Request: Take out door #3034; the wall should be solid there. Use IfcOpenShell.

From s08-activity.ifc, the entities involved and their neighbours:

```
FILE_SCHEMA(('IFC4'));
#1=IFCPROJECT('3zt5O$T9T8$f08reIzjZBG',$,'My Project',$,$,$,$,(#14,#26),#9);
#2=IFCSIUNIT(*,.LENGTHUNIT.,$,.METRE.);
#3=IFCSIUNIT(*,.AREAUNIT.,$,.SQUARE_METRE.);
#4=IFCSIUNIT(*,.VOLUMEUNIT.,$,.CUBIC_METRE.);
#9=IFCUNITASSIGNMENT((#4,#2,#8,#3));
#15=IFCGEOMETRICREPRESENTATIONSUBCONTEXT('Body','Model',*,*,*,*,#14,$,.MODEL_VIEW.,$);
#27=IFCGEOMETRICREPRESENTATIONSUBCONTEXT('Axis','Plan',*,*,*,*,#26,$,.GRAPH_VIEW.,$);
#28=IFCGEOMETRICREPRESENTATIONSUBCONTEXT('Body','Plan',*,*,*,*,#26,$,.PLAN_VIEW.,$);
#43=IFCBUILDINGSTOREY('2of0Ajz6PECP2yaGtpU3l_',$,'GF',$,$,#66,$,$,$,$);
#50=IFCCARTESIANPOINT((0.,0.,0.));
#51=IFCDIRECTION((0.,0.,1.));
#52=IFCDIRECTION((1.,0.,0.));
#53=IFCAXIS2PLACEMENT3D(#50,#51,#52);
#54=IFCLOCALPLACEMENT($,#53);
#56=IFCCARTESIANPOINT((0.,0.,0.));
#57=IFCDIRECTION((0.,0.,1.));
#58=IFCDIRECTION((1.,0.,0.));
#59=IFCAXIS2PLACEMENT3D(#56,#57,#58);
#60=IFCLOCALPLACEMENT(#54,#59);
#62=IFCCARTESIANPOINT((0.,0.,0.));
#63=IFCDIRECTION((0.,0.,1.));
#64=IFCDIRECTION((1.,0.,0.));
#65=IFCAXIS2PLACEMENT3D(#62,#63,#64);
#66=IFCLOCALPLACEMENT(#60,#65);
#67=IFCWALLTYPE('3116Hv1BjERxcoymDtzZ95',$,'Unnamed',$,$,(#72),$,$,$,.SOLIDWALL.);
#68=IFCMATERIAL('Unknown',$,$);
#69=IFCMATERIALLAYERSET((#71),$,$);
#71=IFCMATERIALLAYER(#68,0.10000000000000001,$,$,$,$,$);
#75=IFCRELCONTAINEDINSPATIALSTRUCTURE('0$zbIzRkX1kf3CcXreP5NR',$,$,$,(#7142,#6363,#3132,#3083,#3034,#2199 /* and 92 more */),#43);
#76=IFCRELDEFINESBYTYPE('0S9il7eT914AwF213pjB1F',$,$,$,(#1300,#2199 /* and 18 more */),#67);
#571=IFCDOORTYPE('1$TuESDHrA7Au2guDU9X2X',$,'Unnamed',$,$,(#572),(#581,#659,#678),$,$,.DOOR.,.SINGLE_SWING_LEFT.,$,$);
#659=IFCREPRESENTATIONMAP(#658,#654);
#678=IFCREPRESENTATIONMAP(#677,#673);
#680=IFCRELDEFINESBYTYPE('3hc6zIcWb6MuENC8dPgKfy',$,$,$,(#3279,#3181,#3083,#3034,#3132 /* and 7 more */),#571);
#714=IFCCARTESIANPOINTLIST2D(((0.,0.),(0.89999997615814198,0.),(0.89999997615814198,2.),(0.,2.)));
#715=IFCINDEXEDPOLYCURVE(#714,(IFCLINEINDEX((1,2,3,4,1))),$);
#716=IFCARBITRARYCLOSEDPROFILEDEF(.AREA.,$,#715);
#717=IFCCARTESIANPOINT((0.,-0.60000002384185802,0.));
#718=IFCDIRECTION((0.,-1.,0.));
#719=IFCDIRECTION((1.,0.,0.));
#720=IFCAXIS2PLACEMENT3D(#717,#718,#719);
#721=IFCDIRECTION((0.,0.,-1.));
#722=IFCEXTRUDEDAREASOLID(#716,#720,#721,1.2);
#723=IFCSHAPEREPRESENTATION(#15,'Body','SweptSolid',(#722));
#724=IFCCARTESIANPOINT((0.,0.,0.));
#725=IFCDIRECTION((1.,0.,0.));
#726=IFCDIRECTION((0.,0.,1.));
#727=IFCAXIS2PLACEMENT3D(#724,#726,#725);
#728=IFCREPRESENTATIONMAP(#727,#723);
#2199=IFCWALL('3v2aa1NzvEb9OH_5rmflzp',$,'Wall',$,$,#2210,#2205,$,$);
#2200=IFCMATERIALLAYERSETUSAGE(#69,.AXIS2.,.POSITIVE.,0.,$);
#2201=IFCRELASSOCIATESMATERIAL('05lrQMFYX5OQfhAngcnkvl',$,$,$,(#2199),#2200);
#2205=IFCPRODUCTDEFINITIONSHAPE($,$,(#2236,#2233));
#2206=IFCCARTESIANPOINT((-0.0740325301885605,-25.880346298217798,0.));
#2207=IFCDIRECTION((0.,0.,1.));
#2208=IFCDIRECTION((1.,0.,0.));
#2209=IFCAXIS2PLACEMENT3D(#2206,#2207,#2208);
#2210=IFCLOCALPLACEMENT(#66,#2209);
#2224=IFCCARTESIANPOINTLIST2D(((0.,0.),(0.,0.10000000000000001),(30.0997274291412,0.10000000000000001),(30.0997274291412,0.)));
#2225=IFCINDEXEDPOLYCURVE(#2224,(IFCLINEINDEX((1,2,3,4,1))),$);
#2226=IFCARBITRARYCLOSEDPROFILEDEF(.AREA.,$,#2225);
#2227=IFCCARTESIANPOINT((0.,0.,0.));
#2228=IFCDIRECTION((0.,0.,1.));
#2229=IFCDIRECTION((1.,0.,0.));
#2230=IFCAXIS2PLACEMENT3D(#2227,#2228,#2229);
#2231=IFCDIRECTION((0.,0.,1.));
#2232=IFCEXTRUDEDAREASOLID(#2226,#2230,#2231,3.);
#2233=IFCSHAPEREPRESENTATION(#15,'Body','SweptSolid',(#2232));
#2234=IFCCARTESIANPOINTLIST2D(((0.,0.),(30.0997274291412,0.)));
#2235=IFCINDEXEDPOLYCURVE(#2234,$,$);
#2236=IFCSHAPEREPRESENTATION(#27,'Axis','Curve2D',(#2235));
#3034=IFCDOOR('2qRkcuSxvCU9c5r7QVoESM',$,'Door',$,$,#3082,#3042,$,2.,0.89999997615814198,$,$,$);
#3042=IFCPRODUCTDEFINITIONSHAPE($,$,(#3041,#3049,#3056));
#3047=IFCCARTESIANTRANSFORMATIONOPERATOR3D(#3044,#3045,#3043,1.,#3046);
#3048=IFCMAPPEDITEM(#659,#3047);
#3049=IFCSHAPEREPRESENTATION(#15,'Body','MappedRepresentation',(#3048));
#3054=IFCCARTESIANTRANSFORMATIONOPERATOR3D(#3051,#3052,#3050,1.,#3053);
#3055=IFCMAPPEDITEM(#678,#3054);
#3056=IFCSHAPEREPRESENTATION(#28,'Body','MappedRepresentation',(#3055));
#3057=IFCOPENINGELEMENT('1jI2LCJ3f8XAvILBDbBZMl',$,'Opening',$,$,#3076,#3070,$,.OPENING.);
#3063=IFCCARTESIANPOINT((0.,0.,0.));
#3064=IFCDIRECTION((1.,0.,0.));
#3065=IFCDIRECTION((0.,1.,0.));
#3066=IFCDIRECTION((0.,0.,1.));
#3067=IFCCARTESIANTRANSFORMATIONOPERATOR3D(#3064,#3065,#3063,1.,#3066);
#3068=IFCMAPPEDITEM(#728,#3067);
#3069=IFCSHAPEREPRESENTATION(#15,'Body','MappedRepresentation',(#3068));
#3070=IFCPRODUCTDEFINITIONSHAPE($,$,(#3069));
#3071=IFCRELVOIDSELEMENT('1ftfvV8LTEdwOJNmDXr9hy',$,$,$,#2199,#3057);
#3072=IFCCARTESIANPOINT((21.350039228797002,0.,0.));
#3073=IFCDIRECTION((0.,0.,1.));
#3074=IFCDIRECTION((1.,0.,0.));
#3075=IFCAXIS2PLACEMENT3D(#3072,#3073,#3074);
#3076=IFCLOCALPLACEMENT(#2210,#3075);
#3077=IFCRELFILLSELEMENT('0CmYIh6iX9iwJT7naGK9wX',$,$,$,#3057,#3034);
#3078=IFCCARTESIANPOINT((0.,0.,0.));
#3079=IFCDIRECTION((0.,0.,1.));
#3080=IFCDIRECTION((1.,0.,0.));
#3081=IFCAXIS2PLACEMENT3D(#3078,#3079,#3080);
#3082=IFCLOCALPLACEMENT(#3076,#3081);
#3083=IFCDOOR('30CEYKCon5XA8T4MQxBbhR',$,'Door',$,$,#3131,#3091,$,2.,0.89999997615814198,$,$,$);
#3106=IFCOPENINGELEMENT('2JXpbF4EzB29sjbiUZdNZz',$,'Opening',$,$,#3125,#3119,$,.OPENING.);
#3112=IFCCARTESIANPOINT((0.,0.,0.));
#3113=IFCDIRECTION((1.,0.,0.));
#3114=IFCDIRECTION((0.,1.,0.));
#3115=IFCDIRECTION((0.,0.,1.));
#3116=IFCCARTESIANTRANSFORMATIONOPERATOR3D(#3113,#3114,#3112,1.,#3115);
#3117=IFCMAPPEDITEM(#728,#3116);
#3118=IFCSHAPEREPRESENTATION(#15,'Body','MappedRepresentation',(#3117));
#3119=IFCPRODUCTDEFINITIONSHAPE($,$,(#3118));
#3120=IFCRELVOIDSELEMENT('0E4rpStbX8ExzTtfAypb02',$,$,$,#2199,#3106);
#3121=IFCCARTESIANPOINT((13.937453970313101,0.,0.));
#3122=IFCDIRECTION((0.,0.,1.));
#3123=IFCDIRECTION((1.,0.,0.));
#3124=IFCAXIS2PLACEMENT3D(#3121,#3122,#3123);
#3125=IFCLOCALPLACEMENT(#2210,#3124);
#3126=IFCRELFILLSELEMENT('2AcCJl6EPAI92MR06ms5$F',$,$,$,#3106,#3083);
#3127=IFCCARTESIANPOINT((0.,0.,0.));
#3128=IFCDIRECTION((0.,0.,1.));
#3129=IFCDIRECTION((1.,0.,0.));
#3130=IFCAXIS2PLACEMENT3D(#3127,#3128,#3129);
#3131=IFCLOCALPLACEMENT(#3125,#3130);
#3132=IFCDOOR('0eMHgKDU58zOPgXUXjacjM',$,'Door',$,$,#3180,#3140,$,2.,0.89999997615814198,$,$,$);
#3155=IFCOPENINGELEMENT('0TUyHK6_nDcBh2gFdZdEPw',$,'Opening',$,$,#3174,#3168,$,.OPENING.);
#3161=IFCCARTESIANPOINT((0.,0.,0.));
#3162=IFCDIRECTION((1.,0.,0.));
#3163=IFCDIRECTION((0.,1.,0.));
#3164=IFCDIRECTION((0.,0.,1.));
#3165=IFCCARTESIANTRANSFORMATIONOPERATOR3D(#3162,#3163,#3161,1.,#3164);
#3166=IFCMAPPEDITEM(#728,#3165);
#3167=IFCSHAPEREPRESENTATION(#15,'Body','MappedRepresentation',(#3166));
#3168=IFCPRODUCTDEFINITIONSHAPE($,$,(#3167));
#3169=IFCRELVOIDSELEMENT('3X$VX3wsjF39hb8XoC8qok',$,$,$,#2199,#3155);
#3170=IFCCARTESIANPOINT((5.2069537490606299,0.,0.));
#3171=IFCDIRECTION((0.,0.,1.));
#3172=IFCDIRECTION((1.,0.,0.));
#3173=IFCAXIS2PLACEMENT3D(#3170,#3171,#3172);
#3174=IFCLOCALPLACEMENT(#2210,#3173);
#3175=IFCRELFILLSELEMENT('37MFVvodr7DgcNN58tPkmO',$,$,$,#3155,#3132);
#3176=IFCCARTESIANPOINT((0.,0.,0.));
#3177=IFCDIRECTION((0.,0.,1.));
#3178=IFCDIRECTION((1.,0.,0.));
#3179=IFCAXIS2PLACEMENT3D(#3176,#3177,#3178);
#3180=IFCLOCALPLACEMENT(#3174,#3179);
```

```python
import ifcopenshell
import ifcopenshell.api.feature
import ifcopenshell.api.root
import ifcopenshell.geom
import ifcopenshell.util.shape

model = ifcopenshell.open("s08-activity.ifc")
settings = ifcopenshell.geom.settings()


def volume(element):
    """Net volume in cubic metres, openings subtracted."""
    shape = ifcopenshell.geom.create_shape(settings, element)
    return ifcopenshell.util.shape.get_volume(shape.geometry)


door = model.by_id(3034)
opening = door.FillsVoids[0].RelatingOpeningElement
wall = opening.VoidsElements[0].RelatingBuildingElement
before = volume(wall)

ifcopenshell.api.root.remove_product(model, product=door)
ifcopenshell.api.feature.remove_feature(model, feature=opening)

after = volume(wall)

print(f"wall volume {before:.3f} -> {after:.3f} m3")

model.write("s08-activity_edited.ifc")
```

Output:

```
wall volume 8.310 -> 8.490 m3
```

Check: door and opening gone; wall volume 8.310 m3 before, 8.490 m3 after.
